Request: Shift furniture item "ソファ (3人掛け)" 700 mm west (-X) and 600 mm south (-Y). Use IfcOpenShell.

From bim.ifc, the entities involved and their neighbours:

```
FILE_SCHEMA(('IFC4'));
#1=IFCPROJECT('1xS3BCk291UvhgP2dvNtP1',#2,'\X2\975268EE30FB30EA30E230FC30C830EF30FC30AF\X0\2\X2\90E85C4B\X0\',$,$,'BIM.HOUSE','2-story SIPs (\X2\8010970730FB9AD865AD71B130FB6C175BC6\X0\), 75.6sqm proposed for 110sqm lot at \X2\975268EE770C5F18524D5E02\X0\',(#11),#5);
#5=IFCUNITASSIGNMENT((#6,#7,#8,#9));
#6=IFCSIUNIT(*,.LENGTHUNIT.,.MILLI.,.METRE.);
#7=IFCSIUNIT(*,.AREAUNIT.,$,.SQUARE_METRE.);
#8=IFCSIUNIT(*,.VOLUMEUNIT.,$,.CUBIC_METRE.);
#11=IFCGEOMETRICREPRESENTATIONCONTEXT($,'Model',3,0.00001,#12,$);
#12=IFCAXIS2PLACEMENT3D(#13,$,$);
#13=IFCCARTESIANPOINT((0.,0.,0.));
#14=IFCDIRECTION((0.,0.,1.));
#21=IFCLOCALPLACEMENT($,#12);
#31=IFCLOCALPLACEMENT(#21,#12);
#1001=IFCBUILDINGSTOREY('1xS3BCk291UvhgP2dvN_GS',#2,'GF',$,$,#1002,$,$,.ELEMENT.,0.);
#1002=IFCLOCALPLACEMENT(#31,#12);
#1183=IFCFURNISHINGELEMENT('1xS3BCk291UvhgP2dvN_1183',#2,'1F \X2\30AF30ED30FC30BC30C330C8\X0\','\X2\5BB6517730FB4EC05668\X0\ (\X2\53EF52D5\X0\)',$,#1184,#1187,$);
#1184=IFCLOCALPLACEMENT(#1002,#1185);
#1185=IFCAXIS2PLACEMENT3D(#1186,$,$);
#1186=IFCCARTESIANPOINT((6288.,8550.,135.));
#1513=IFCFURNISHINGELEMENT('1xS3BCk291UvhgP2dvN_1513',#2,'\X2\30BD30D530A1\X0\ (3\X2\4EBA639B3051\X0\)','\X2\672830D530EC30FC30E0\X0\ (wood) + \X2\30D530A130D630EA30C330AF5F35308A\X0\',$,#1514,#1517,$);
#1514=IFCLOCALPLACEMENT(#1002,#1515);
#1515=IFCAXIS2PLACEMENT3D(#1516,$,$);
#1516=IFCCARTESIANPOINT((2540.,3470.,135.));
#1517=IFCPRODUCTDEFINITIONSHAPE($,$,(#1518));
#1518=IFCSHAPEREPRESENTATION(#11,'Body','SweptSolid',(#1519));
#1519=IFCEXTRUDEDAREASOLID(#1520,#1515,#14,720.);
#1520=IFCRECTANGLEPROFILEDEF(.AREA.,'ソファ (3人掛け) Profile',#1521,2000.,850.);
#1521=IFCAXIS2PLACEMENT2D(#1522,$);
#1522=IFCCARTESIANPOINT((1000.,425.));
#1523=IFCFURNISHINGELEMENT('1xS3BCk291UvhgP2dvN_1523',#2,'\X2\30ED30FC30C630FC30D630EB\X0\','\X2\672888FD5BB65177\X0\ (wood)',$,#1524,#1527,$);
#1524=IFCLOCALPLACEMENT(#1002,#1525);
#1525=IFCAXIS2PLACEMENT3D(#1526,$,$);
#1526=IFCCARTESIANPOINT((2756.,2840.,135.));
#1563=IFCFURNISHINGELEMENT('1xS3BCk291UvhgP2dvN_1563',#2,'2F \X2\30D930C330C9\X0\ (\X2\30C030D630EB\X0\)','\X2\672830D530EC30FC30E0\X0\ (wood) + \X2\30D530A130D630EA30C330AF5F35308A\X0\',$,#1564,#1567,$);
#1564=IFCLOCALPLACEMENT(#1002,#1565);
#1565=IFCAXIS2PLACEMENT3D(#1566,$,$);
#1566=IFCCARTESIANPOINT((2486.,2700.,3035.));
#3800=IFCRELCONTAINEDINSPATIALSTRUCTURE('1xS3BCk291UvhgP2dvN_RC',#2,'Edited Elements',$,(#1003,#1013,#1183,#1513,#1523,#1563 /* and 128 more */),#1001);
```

```python
import ifcopenshell
import ifcopenshell.api.geometry
import ifcopenshell.util.placement

model = ifcopenshell.open("bim.ifc")

item = model.by_guid("1xS3BCk291UvhgP2dvN_1513")
matrix = ifcopenshell.util.placement.get_local_placement(item.ObjectPlacement)
matrix[0, 3] -= 700.0
matrix[1, 3] -= 600.0
ifcopenshell.api.geometry.edit_object_placement(model, product=item, matrix=matrix, is_si=False)

print(ifcopenshell.util.placement.get_local_placement(item.ObjectPlacement).round(3) + 0.0)

model.write("bim_v2.ifc")
```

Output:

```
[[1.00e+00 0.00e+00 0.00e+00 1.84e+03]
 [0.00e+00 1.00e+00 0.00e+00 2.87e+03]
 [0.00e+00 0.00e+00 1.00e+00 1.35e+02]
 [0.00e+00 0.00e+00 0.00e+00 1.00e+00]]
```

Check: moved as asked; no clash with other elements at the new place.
